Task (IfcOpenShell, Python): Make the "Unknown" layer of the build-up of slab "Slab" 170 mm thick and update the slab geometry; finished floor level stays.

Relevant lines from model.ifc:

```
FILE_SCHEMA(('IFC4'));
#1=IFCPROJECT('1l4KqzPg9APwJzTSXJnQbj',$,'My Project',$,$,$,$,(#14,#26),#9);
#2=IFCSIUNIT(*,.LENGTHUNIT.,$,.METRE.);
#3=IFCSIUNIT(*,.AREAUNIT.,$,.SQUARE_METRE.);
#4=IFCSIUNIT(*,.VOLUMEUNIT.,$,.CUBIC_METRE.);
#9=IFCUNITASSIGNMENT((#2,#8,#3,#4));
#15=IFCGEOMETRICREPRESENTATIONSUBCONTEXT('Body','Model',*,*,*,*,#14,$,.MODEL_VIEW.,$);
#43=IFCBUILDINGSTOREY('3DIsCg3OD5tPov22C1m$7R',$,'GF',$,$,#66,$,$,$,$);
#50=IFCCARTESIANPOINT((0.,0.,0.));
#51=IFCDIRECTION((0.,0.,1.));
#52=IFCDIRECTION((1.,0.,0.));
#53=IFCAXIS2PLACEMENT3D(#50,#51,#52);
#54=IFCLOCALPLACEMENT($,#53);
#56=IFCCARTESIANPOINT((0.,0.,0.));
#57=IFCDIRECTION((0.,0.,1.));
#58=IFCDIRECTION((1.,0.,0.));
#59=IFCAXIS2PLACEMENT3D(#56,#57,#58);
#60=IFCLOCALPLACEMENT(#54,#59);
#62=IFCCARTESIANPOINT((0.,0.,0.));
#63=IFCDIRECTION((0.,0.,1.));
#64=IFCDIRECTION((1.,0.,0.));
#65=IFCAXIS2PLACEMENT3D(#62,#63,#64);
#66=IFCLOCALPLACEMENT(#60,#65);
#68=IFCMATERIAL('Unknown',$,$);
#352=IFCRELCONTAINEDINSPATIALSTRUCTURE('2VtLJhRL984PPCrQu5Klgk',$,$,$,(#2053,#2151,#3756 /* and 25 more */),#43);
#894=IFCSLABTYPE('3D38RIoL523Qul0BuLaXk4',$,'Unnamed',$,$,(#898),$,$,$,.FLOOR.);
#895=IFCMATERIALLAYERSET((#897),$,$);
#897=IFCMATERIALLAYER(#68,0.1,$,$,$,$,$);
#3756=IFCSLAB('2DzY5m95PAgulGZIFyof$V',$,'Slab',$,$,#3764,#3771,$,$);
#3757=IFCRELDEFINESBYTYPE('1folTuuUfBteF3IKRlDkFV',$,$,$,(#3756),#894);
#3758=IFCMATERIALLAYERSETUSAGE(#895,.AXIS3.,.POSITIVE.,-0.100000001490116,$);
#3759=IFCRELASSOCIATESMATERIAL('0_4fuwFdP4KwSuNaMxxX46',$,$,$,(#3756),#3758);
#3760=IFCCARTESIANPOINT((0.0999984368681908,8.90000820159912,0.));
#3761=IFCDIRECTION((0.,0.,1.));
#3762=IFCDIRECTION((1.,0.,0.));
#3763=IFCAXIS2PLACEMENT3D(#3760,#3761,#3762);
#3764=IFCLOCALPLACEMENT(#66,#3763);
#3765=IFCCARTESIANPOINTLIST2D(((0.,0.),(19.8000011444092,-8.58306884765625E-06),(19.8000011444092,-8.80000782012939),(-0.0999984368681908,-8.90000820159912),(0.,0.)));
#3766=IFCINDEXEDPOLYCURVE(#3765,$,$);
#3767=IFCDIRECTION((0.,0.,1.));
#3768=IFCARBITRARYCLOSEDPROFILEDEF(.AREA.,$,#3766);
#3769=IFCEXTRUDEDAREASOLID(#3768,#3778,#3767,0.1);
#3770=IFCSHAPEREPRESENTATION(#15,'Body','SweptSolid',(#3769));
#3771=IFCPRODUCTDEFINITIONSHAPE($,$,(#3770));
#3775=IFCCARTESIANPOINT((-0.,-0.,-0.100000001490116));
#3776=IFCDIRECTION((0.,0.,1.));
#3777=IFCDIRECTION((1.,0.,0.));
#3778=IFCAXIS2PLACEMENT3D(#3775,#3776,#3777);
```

```python
import ifcopenshell
import ifcopenshell.util.element
import ifcopenshell.util.representation
import ifcopenshell.util.unit

model = ifcopenshell.open("model.ifc")
unit_scale = ifcopenshell.util.unit.calculate_unit_scale(model)

layer_set = model.by_id(895)
layer = next(l for l in layer_set.MaterialLayers if l.Material and l.Material.Name == "Unknown")
change = 0.17 / unit_scale - layer.LayerThickness
layer.LayerThickness += change

# Geometry does not follow the layer set by itself.
slabs = [e for e in ifcopenshell.util.element.get_elements_by_material(model, layer_set) if e.is_a("IfcSlab")]
for slab in sorted(slabs, key=lambda e: e.id()):
    body = ifcopenshell.util.representation.get_representation(slab, "Model", "Body")
    solid = body.Items[0]
    old_depth = solid.Depth
    solid.Depth += change
    # Extruded upwards: lower the start of the extrusion so the top stays.
    x, y, z = solid.Position.Location.Coordinates
    solid.Position.Location = model.createIfcCartesianPoint((x, y, z - change))
    print(slab.id(), f"{old_depth:g} -> {solid.Depth:g}")

# The layers are counted up from the underside, which has moved.
for usage in {ifcopenshell.util.element.get_material(slab) for slab in slabs}:
    usage.OffsetFromReferenceLine -= change

model.write("model_rev.ifc")
```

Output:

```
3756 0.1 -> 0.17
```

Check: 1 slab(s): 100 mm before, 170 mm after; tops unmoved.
